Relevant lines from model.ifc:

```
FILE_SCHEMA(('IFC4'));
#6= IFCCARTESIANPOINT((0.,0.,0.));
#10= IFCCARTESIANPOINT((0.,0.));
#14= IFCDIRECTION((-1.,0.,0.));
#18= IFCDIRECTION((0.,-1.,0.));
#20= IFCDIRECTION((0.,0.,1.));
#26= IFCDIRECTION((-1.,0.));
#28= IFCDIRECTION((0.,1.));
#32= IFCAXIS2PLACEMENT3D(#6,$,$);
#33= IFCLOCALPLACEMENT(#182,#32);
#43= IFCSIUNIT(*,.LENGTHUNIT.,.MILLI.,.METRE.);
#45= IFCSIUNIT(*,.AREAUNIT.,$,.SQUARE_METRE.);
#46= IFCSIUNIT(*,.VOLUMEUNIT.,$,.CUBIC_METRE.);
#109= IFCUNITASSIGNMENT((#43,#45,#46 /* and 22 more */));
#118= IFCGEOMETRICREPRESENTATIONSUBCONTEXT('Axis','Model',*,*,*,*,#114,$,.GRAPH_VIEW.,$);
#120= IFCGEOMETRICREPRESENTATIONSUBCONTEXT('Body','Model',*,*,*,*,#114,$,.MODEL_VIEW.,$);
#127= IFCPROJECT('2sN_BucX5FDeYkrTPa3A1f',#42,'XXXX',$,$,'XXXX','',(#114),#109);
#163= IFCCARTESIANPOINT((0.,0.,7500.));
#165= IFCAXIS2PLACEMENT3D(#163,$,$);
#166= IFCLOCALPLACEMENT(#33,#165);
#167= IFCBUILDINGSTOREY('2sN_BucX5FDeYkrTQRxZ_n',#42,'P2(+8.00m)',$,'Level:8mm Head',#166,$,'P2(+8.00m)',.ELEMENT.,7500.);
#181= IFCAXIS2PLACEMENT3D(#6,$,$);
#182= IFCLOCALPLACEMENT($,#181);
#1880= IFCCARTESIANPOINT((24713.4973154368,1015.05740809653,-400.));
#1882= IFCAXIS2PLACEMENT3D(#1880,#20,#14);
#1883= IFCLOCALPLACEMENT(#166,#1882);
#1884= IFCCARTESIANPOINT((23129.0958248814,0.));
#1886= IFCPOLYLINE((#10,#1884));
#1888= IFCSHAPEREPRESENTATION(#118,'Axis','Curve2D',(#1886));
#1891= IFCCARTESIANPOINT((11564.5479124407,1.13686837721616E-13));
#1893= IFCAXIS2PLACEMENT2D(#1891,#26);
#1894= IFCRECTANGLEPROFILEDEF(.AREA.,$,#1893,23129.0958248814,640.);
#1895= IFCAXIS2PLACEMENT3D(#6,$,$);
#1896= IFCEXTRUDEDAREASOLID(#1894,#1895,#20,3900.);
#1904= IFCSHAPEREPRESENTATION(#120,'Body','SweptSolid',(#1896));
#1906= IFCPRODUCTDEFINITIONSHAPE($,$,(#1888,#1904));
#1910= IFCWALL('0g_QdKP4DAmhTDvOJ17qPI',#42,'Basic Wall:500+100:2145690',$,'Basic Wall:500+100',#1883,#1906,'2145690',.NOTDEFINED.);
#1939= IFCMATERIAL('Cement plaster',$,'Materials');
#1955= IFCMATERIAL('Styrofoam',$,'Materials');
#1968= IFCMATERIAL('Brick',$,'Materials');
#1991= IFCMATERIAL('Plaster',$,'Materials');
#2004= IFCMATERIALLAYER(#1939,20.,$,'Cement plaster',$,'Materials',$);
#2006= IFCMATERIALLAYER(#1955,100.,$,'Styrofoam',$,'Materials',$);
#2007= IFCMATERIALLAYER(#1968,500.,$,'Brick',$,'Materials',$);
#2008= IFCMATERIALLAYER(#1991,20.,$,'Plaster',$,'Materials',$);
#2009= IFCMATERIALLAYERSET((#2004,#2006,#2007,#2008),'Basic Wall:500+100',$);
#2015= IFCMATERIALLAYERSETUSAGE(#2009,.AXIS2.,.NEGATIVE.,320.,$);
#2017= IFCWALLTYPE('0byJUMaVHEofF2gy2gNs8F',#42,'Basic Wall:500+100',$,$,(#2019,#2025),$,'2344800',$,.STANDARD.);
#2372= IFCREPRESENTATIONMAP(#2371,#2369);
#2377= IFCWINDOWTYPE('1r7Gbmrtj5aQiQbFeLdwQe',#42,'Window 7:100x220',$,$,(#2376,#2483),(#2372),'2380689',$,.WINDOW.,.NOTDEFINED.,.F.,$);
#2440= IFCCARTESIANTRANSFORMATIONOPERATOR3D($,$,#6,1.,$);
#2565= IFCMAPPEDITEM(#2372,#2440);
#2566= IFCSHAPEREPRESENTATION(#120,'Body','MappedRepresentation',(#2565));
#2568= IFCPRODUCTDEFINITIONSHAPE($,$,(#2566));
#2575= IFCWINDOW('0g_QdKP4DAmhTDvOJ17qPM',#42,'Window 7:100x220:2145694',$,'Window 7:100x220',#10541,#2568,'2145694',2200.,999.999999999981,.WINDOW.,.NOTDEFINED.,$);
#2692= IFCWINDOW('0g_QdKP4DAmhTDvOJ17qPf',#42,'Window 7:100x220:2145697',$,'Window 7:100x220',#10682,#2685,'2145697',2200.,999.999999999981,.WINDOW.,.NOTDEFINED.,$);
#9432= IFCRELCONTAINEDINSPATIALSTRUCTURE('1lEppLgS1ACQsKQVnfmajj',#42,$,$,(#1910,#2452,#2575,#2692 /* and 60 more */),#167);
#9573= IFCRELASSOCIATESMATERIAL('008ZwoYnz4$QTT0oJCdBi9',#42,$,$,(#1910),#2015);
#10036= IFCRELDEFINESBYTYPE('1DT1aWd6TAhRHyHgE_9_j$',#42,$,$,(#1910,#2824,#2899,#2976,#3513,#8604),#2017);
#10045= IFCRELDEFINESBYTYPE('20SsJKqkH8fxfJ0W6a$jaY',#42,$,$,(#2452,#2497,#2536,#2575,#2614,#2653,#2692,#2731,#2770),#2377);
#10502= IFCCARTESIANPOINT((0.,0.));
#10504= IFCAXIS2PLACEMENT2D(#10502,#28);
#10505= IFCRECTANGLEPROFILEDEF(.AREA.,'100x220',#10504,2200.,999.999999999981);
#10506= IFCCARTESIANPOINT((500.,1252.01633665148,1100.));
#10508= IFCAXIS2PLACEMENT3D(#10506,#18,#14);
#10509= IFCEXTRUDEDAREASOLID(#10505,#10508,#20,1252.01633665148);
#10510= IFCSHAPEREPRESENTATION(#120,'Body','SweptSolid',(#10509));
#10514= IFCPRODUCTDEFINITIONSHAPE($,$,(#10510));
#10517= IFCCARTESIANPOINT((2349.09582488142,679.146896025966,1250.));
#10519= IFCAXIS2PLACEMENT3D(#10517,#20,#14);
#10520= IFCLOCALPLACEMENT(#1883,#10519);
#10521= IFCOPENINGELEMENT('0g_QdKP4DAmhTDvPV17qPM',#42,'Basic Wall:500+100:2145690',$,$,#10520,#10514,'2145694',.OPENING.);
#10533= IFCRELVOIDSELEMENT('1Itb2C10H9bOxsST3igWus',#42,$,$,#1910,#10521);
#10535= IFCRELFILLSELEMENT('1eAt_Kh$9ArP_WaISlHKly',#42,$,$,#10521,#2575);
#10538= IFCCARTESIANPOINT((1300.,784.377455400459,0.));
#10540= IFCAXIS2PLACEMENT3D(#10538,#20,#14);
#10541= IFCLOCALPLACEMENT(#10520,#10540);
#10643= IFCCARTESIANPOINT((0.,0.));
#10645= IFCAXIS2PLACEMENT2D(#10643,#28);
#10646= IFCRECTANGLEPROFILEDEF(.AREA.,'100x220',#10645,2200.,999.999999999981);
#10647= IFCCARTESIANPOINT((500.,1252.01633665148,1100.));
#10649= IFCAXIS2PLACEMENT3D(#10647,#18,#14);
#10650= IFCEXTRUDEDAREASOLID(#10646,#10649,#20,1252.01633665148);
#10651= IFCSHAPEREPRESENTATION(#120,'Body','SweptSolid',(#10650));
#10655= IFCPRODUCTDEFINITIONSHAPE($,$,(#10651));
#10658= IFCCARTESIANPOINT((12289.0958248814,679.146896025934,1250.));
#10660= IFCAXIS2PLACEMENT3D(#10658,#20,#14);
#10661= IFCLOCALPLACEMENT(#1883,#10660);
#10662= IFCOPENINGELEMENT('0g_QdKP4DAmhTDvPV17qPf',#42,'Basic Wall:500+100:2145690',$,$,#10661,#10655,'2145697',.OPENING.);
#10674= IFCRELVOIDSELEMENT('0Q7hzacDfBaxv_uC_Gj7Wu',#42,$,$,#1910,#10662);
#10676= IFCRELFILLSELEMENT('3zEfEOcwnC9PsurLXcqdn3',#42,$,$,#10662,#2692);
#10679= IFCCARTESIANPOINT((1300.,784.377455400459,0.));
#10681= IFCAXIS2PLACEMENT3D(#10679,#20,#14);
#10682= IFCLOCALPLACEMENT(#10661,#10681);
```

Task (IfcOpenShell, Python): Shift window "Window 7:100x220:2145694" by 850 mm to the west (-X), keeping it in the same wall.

```python
import ifcopenshell
import ifcopenshell.api.geometry
import ifcopenshell.util.placement

model = ifcopenshell.open("model.ifc")

window = model.by_guid("0g_QdKP4DAmhTDvOJ17qPM")
opening = window.FillsVoids[0].RelatingOpeningElement
wall = opening.VoidsElements[0].RelatingBuildingElement

wall_matrix = ifcopenshell.util.placement.get_local_placement(wall.ObjectPlacement)
shift = wall_matrix[:3, 0] * 850.0
before = ifcopenshell.util.placement.get_local_placement(window.ObjectPlacement)[:3, 3].copy()

# The window is placed relative to its opening, so it follows when the opening moves.
matrix = ifcopenshell.util.placement.get_local_placement(opening.ObjectPlacement)
matrix[:3, 3] += shift
ifcopenshell.api.geometry.edit_object_placement(
    model, product=opening, matrix=matrix, is_si=False, should_transform_children=True
)

after = ifcopenshell.util.placement.get_local_placement(window.ObjectPlacement)[:3, 3]
print("window moved by", (after - before).round(3) + 0.0)

model.write("model_v2.ifc")
```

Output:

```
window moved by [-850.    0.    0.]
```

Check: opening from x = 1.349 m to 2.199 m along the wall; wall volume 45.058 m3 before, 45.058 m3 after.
